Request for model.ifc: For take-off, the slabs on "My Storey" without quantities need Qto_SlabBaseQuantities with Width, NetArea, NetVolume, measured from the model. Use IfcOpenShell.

First a look at what the model holds.

```python
import ifcopenshell
import ifcopenshell.util.element
import ifcopenshell.util.unit

model = ifcopenshell.open("model.ifc")
print(model.schema)
for unit_type in ("LENGTHUNIT", "AREAUNIT", "VOLUMEUNIT"):
    print(unit_type, ifcopenshell.util.unit.calculate_unit_scale(model, unit_type))
storey = next(s for s in model.by_type("IfcBuildingStorey") if s.Name == "My Storey")
slabs = [e for e in ifcopenshell.util.element.get_decomposition(storey) if e.is_a("IfcSlab")]
for e in sorted(slabs, key=lambda e: e.id()):
    print(e.id(), e.is_a(), e.Name, list(ifcopenshell.util.element.get_psets(e, qtos_only=True)), sep=" | ")
```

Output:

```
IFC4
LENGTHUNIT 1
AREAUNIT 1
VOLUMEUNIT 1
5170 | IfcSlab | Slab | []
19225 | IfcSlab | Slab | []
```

```python
import ifcopenshell
import ifcopenshell.api.pset
import ifcopenshell.geom
import ifcopenshell.util.element
import ifcopenshell.util.shape
import ifcopenshell.util.unit

model = ifcopenshell.open("model.ifc")
unit_scale = ifcopenshell.util.unit.calculate_unit_scale(model)
area_scale = ifcopenshell.util.unit.calculate_unit_scale(model, "AREAUNIT")
volume_scale = ifcopenshell.util.unit.calculate_unit_scale(model, "VOLUMEUNIT")
settings = ifcopenshell.geom.settings()

storey = next(s for s in model.by_type("IfcBuildingStorey") if s.Name == "My Storey")
slabs = [e for e in ifcopenshell.util.element.get_decomposition(storey) if e.is_a("IfcSlab")]

for e in sorted(slabs, key=lambda e: e.id()):
    if ifcopenshell.util.element.get_psets(e, qtos_only=True, should_inherit=False):
        continue
    # Geometry comes back in metres, in the element's own axes.
    shape = ifcopenshell.geom.create_shape(settings, e)
    values = {
        "Width": ifcopenshell.util.shape.get_z(shape.geometry) / unit_scale,
        "NetArea": ifcopenshell.util.shape.get_footprint_area(shape.geometry) / area_scale,
        "NetVolume": ifcopenshell.util.shape.get_volume(shape.geometry) / volume_scale,
    }
    qto = ifcopenshell.api.pset.add_qto(model, product=e, name="Qto_SlabBaseQuantities")
    ifcopenshell.api.pset.edit_qto(model, qto=qto, properties=values)
    print(e.id(), {k: round(v, 3) for k, v in values.items()})

model.write("model_v2.ifc")
```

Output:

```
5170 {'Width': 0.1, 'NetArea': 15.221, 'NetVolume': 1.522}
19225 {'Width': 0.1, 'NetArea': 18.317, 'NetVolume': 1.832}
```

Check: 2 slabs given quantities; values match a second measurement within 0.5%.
